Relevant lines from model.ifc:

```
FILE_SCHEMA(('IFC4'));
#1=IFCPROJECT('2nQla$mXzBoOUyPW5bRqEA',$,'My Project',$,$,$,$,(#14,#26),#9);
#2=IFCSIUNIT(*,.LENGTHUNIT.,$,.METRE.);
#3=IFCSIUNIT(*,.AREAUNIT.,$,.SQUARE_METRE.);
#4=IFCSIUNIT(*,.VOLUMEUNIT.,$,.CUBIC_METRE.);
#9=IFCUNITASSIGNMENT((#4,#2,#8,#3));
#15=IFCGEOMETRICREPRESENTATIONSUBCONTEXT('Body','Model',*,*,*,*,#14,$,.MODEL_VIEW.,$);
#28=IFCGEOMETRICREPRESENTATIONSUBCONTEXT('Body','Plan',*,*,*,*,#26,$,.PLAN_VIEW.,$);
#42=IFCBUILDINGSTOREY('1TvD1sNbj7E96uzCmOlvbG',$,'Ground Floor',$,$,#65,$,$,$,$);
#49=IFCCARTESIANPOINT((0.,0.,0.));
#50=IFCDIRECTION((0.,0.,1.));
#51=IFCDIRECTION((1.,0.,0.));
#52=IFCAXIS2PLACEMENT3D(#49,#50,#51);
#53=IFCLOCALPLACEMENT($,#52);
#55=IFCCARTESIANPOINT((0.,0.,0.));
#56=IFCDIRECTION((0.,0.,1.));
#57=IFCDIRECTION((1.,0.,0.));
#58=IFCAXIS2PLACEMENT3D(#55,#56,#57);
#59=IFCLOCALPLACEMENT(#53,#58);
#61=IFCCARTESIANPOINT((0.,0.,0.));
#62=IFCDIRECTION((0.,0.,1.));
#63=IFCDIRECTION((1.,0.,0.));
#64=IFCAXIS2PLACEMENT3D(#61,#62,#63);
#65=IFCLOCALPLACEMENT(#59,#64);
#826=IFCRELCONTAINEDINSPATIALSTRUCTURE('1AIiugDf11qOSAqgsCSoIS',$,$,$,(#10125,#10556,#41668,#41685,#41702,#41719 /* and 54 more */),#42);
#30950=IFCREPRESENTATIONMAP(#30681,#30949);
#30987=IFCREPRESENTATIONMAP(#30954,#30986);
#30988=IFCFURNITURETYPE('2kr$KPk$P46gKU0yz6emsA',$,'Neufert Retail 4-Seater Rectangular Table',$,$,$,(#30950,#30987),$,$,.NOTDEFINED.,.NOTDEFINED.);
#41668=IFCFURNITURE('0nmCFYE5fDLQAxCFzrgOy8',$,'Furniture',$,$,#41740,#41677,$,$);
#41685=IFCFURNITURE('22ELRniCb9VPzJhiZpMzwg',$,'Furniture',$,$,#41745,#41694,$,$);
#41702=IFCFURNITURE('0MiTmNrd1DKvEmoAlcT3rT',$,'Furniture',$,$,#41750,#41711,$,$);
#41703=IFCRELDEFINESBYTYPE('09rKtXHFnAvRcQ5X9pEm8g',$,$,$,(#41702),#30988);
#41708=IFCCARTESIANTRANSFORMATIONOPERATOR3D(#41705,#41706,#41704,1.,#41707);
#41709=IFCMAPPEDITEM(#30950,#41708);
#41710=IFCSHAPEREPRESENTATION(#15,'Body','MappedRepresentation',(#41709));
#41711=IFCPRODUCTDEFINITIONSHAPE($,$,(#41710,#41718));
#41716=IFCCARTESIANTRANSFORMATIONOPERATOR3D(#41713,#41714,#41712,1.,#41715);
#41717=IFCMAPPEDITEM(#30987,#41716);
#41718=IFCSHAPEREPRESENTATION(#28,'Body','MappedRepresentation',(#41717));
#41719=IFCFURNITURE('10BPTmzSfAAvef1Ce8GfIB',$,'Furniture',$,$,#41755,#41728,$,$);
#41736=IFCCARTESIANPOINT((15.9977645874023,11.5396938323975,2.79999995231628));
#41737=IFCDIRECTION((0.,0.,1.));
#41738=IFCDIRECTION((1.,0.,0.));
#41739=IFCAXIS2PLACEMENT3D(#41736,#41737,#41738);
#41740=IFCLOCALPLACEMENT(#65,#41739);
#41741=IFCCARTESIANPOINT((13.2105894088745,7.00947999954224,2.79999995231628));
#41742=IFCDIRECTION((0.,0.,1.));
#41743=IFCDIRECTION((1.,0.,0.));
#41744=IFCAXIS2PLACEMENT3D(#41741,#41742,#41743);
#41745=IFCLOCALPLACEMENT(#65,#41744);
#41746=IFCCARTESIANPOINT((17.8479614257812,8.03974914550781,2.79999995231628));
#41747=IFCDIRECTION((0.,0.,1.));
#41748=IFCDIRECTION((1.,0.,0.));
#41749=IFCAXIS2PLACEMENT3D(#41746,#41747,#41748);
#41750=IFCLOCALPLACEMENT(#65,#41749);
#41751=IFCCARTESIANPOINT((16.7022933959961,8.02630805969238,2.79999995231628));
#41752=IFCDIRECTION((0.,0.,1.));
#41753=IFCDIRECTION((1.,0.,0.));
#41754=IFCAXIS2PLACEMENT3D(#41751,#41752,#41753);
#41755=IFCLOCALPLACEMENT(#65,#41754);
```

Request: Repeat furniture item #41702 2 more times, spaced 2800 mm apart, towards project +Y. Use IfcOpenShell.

```python
import numpy as np
import ifcopenshell
import ifcopenshell.api.geometry
import ifcopenshell.api.root
import ifcopenshell.util.element
import ifcopenshell.util.placement
import ifcopenshell.util.unit

model = ifcopenshell.open("model.ifc")
unit_scale = ifcopenshell.util.unit.calculate_unit_scale(model)

source = model.by_guid("0MiTmNrd1DKvEmoAlcT3rT")
base = ifcopenshell.util.placement.get_local_placement(source.ObjectPlacement)
step = np.array([0.0, 1.0, 0.0]) * 2.8 / unit_scale

for i in range(1, 3):
    copy = ifcopenshell.api.root.copy_class(model, product=source)
    copy.Representation = ifcopenshell.util.element.copy_deep(
        model, source.Representation, exclude=["IfcGeometricRepresentationContext", "IfcRepresentationMap"]
    )
    matrix = base.copy()
    matrix[:3, 3] += i * step
    print("added at", matrix[:3, 3].round(3) + 0.0)
    ifcopenshell.api.geometry.edit_object_placement(model, product=copy, matrix=matrix, is_si=False)

model.write("model-out.ifc")
```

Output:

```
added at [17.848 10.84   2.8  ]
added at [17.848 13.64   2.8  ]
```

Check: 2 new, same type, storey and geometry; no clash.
